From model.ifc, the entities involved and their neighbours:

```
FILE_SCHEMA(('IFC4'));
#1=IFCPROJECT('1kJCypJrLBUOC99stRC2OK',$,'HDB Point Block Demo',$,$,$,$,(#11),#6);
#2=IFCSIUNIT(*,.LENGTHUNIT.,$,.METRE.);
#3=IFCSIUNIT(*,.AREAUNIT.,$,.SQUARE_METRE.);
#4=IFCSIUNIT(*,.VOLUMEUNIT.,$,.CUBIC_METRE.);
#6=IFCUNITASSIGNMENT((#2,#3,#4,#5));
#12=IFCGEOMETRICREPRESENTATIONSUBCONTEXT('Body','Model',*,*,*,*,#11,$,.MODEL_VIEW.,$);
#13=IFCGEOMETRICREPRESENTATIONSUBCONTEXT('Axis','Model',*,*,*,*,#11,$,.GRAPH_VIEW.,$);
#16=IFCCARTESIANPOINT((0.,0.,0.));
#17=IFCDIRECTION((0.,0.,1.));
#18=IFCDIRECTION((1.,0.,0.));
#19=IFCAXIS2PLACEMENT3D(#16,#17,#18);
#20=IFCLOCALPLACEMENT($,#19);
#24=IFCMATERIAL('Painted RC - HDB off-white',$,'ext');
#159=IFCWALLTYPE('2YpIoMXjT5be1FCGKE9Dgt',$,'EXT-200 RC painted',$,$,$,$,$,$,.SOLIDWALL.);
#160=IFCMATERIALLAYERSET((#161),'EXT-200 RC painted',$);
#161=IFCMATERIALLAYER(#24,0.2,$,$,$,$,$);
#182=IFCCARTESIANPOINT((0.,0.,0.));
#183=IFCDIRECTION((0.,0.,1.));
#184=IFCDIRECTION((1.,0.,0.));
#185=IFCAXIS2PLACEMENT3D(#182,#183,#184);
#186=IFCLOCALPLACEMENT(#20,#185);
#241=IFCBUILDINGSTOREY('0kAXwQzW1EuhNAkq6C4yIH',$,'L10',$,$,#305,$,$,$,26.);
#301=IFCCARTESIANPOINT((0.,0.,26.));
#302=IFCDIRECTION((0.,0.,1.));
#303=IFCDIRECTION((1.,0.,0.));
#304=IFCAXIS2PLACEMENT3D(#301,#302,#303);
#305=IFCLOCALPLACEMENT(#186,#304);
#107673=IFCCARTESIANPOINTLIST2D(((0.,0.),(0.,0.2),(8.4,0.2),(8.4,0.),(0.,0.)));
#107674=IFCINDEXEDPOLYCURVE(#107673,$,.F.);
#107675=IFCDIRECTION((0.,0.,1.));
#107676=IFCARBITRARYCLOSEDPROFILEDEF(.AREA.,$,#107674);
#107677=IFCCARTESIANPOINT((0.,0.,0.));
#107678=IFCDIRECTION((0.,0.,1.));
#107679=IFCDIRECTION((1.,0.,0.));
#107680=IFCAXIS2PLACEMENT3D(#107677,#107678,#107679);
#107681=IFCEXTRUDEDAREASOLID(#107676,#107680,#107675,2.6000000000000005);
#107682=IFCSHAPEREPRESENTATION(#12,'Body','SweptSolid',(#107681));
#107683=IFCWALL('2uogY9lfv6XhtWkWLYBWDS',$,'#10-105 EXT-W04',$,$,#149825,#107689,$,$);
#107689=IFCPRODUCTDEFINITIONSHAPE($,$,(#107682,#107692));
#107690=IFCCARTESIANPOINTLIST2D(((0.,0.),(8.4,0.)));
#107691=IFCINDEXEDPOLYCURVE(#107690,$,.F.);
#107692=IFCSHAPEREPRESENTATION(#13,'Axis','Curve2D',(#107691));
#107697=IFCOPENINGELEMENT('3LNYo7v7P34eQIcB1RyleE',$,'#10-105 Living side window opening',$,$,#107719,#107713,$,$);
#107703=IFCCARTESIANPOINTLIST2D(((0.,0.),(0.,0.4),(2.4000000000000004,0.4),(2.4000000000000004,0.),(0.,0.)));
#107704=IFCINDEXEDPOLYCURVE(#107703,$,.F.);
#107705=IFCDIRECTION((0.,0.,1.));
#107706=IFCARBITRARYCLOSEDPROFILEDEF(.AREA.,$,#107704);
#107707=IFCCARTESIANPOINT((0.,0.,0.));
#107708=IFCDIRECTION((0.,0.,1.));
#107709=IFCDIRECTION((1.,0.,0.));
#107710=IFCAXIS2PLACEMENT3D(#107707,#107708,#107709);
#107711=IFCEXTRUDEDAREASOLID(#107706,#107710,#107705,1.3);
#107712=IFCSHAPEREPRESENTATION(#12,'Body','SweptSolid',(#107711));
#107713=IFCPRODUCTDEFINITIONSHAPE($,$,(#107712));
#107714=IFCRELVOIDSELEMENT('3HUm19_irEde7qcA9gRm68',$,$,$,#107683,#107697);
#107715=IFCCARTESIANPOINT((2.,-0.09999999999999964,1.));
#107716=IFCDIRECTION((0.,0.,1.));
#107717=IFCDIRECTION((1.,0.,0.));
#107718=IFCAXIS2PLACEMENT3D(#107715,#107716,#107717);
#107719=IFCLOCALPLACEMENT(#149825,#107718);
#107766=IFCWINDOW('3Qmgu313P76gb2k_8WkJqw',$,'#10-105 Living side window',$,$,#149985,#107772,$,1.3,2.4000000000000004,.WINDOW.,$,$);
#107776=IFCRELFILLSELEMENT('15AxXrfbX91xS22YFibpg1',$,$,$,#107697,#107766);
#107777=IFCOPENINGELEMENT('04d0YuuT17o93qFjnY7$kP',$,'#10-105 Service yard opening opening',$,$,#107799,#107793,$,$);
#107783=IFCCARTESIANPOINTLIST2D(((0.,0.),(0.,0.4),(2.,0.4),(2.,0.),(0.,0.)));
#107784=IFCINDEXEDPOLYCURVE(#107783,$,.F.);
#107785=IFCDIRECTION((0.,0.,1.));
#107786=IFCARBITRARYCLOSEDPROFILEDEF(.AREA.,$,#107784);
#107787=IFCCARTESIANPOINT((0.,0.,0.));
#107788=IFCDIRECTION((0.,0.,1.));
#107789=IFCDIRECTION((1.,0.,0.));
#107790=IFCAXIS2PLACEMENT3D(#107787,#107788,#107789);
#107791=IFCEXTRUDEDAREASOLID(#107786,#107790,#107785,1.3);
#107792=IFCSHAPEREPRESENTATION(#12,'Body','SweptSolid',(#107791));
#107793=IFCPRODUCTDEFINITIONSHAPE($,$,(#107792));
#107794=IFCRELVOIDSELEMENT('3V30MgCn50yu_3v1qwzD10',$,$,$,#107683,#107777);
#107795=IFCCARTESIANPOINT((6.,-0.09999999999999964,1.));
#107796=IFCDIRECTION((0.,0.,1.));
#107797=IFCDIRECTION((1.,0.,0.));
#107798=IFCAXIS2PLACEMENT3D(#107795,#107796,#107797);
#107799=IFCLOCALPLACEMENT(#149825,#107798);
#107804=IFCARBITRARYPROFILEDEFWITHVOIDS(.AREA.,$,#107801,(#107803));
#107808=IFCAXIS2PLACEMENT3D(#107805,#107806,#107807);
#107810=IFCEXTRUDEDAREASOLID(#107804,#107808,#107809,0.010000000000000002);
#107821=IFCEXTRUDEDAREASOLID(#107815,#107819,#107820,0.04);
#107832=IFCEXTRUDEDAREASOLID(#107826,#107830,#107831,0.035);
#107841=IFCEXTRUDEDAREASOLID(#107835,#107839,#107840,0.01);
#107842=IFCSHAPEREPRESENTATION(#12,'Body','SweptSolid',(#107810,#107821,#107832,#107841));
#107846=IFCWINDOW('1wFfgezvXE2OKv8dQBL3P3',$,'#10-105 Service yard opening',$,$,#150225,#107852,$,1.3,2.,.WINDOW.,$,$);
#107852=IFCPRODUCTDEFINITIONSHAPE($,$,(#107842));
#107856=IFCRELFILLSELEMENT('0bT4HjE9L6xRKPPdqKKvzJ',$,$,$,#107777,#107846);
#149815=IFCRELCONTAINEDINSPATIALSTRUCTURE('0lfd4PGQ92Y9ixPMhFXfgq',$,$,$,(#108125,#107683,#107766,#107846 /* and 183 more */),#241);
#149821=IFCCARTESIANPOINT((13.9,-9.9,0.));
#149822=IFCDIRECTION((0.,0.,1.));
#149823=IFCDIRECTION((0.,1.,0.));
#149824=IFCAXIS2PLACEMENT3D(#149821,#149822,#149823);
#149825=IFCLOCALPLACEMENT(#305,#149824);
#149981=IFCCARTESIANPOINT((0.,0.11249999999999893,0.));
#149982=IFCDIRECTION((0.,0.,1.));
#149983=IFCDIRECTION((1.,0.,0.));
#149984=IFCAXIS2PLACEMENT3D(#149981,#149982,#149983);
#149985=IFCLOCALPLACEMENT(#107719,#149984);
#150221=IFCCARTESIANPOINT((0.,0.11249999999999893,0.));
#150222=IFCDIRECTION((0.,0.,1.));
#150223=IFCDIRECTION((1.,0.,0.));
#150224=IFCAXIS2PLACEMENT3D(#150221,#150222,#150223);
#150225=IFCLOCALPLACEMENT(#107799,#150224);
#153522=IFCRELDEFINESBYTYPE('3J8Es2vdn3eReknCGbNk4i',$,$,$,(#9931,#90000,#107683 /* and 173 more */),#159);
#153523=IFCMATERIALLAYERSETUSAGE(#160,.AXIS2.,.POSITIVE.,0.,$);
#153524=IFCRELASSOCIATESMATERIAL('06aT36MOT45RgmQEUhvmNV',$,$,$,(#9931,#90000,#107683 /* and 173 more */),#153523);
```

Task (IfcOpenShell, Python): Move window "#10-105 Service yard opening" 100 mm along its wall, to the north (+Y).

```python
import ifcopenshell
import ifcopenshell.api.geometry
import ifcopenshell.util.placement
import ifcopenshell.util.unit

model = ifcopenshell.open("model.ifc")
unit_scale = ifcopenshell.util.unit.calculate_unit_scale(model)

window = model.by_guid("1wFfgezvXE2OKv8dQBL3P3")
opening = window.FillsVoids[0].RelatingOpeningElement
wall = opening.VoidsElements[0].RelatingBuildingElement

wall_matrix = ifcopenshell.util.placement.get_local_placement(wall.ObjectPlacement)
shift = wall_matrix[:3, 0] * 0.1 / unit_scale
before = ifcopenshell.util.placement.get_local_placement(window.ObjectPlacement)[:3, 3].copy()

# The window is placed relative to its opening, so it follows when the opening moves.
matrix = ifcopenshell.util.placement.get_local_placement(opening.ObjectPlacement)
matrix[:3, 3] += shift
ifcopenshell.api.geometry.edit_object_placement(
    model, product=opening, matrix=matrix, is_si=False, should_transform_children=True
)

after = ifcopenshell.util.placement.get_local_placement(window.ObjectPlacement)[:3, 3]
print("window moved by", (after - before).round(3) + 0.0)

model.write("model_v2.ifc")
```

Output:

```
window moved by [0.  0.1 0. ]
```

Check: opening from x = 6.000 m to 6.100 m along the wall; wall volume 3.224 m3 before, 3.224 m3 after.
